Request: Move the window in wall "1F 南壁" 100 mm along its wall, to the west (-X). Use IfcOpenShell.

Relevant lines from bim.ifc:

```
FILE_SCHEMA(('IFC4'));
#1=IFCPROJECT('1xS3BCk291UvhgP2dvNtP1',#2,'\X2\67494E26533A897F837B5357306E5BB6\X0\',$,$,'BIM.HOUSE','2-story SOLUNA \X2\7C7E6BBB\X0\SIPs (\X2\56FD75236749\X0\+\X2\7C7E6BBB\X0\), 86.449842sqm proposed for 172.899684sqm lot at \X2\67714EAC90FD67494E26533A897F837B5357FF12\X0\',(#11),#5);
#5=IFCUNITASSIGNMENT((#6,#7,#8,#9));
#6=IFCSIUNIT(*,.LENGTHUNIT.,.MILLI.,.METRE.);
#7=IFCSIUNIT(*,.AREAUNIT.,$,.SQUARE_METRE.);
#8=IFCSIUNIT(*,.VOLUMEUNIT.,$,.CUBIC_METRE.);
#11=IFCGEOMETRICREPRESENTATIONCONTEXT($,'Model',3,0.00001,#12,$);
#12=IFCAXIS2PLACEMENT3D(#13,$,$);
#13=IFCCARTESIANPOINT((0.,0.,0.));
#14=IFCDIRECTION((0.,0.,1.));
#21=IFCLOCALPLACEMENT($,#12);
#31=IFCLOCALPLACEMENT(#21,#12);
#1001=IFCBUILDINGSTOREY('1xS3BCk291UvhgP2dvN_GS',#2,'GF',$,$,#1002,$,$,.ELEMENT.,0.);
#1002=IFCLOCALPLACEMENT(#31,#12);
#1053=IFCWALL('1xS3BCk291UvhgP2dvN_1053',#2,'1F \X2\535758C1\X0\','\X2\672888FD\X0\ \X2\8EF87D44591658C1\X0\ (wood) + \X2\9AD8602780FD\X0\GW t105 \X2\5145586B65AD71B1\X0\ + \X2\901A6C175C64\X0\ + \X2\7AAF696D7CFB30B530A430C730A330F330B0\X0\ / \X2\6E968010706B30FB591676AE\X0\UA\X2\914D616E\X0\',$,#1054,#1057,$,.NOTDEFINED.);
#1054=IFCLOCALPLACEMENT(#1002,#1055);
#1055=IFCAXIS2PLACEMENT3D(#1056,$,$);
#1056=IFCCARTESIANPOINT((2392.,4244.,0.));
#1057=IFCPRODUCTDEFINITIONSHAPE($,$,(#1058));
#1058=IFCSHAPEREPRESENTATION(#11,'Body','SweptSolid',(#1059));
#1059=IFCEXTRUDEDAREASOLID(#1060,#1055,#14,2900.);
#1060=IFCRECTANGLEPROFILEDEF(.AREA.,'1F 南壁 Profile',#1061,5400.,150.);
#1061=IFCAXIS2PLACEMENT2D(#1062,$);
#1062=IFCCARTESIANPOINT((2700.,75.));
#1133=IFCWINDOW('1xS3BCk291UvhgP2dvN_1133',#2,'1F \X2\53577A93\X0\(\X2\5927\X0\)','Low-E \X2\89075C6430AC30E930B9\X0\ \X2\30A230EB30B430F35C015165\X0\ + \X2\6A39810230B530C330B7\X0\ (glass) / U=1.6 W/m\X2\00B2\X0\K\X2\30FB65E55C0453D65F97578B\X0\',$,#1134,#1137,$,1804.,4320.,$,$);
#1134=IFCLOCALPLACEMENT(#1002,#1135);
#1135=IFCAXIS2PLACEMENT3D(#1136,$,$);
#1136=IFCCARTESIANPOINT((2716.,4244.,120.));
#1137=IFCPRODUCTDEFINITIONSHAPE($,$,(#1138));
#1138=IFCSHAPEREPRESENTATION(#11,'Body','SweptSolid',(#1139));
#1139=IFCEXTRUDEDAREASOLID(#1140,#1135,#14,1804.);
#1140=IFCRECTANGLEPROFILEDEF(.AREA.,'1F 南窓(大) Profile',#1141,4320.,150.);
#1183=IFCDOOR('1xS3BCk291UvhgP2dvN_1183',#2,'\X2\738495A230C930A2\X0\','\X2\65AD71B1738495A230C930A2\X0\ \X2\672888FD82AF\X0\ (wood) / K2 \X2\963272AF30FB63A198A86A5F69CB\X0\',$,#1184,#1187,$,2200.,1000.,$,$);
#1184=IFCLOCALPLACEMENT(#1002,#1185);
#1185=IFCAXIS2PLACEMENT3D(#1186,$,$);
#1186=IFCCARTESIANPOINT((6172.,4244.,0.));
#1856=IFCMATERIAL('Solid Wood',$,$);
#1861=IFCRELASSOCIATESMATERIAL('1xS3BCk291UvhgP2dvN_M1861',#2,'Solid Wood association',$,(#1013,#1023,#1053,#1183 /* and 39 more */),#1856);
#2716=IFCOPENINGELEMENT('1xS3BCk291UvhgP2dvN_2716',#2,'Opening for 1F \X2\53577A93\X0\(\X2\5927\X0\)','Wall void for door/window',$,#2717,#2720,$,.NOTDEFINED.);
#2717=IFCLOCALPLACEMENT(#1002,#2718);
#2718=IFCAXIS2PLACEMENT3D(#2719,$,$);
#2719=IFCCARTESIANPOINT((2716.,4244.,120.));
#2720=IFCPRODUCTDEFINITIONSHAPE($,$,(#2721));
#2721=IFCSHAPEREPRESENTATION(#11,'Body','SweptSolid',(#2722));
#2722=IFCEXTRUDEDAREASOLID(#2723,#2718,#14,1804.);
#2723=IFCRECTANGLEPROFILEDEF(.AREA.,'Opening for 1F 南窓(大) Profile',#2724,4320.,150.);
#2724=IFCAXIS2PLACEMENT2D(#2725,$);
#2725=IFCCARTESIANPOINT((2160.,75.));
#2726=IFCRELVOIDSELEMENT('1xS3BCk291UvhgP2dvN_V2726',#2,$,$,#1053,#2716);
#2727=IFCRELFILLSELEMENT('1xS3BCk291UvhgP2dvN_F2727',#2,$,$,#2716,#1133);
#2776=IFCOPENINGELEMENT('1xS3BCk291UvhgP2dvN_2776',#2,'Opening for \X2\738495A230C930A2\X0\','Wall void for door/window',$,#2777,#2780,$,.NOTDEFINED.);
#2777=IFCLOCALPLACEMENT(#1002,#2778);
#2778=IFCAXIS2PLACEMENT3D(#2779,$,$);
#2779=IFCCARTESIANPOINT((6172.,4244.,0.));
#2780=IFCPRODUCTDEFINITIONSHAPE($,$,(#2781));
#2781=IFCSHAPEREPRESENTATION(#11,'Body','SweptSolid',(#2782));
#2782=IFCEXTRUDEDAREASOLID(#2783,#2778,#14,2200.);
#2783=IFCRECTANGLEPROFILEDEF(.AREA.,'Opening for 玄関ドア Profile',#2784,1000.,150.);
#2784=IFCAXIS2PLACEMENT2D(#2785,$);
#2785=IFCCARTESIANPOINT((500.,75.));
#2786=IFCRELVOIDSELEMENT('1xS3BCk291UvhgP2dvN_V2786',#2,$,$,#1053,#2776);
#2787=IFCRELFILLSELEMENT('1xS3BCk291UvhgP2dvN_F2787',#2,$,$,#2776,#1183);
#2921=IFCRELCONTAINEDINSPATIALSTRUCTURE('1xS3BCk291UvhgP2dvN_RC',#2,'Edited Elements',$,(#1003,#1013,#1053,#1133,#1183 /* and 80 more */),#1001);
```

```python
import ifcopenshell
import ifcopenshell.api.geometry
import ifcopenshell.util.placement
import ifcopenshell.util.unit

model = ifcopenshell.open("bim.ifc")
unit_scale = ifcopenshell.util.unit.calculate_unit_scale(model)

window = model.by_guid("1xS3BCk291UvhgP2dvN_1133")
opening = window.FillsVoids[0].RelatingOpeningElement
wall = opening.VoidsElements[0].RelatingBuildingElement

wall_matrix = ifcopenshell.util.placement.get_local_placement(wall.ObjectPlacement)
shift = wall_matrix[:3, 0] * -0.1 / unit_scale
before = ifcopenshell.util.placement.get_local_placement(window.ObjectPlacement)[:3, 3].copy()

# The window is not placed relative to its opening, so move both.
for product in (opening, window):
    matrix = ifcopenshell.util.placement.get_local_placement(product.ObjectPlacement)
    matrix[:3, 3] += shift
    ifcopenshell.api.geometry.edit_object_placement(model, product=product, matrix=matrix, is_si=False)

after = ifcopenshell.util.placement.get_local_placement(window.ObjectPlacement)[:3, 3]
print("window moved by", (after - before).round(3) + 0.0)

model.write("bim-out.ifc")
```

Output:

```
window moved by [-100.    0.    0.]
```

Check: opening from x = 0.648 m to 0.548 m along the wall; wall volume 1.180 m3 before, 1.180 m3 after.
